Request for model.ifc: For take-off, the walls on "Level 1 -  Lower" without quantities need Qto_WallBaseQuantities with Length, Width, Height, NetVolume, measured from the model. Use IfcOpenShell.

First a look at what the model holds.

```python
import ifcopenshell
import ifcopenshell.util.element
import ifcopenshell.util.unit

model = ifcopenshell.open("model.ifc")
print(model.schema)
for unit_type in ("LENGTHUNIT", "AREAUNIT", "VOLUMEUNIT"):
    print(unit_type, ifcopenshell.util.unit.calculate_unit_scale(model, unit_type))
storey = next(s for s in model.by_type("IfcBuildingStorey") if s.Name == "Level 1 -  Lower")
walls = [e for e in ifcopenshell.util.element.get_decomposition(storey) if e.is_a("IfcWall")]
for e in sorted(walls, key=lambda e: e.id()):
    print(e.id(), e.is_a(), e.Name, list(ifcopenshell.util.element.get_psets(e, qtos_only=True)), sep=" | ")
```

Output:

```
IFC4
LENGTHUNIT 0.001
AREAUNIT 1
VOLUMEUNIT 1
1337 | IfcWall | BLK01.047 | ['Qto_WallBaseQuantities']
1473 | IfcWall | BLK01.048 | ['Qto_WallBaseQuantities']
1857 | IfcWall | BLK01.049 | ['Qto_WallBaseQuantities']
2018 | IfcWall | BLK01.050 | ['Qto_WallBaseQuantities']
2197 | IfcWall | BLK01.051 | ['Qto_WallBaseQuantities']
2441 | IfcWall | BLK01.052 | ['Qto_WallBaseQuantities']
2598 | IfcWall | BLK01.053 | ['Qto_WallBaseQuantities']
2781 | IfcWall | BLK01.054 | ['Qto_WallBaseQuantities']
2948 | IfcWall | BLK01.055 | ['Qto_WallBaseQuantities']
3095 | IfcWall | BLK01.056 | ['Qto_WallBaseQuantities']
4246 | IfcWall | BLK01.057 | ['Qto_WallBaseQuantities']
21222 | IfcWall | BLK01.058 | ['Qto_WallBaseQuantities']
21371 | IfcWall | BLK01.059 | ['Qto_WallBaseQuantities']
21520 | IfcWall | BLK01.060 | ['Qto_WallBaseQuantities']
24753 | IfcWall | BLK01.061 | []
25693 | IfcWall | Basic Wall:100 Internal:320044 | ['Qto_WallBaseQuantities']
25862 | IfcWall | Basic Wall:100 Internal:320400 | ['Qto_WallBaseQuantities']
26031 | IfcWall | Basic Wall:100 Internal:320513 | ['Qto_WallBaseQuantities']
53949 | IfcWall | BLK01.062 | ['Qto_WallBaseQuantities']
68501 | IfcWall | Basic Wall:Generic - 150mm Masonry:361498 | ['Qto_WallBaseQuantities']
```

```python
import ifcopenshell
import ifcopenshell.api.pset
import ifcopenshell.geom
import ifcopenshell.util.element
import ifcopenshell.util.shape
import ifcopenshell.util.unit

model = ifcopenshell.open("model.ifc")
unit_scale = ifcopenshell.util.unit.calculate_unit_scale(model)
volume_scale = ifcopenshell.util.unit.calculate_unit_scale(model, "VOLUMEUNIT")
settings = ifcopenshell.geom.settings()

storey = next(s for s in model.by_type("IfcBuildingStorey") if s.Name == "Level 1 -  Lower")
walls = [e for e in ifcopenshell.util.element.get_decomposition(storey) if e.is_a("IfcWall")]

for e in sorted(walls, key=lambda e: e.id()):
    if ifcopenshell.util.element.get_psets(e, qtos_only=True, should_inherit=False):
        continue
    # Geometry comes back in metres, in the element's own axes.
    shape = ifcopenshell.geom.create_shape(settings, e)
    values = {
        "Length": ifcopenshell.util.shape.get_x(shape.geometry) / unit_scale,
        "Width": ifcopenshell.util.shape.get_y(shape.geometry) / unit_scale,
        "Height": ifcopenshell.util.shape.get_z(shape.geometry) / unit_scale,
        "NetVolume": ifcopenshell.util.shape.get_volume(shape.geometry) / volume_scale,
    }
    qto = ifcopenshell.api.pset.add_qto(model, product=e, name="Qto_WallBaseQuantities")
    ifcopenshell.api.pset.edit_qto(model, qto=qto, properties=values)
    print(e.id(), {k: round(v, 3) for k, v in values.items()})

model.write("model_v2.ifc")
```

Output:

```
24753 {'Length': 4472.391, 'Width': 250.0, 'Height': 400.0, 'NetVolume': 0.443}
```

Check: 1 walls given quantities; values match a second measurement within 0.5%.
